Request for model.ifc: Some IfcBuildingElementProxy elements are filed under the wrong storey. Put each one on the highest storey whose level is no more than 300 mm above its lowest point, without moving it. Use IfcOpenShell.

First a look at what the model holds.

```python
import ifcopenshell
import ifcopenshell.util.element
import ifcopenshell.util.placement

model = ifcopenshell.open("model.ifc")
print(model.schema)
for storey in model.by_type("IfcBuildingStorey"):
    level = ifcopenshell.util.placement.get_storey_elevation(storey)
    count = sum(e.is_a("IfcBuildingElementProxy") for e in ifcopenshell.util.element.get_contained(storey))
    print(storey.id(), storey.Name, round(level, 3), count, sep=" | ")
```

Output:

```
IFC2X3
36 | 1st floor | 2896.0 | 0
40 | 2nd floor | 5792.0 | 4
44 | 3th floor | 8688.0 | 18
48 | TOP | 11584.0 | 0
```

```python
import ifcopenshell
import ifcopenshell.api.spatial
import ifcopenshell.geom
import ifcopenshell.util.element
import ifcopenshell.util.placement
import ifcopenshell.util.shape
import ifcopenshell.util.unit

model = ifcopenshell.open("model.ifc")
unit_scale = ifcopenshell.util.unit.calculate_unit_scale(model)
settings = ifcopenshell.geom.settings()

levels = sorted(
    ((ifcopenshell.util.placement.get_storey_elevation(s) * unit_scale, s) for s in model.by_type("IfcBuildingStorey")),
    key=lambda pair: pair[0],
)

for e in model.by_type("IfcBuildingElementProxy"):
    current = e.ContainedInStructure[0].RelatingStructure if e.ContainedInStructure else None
    if current is None or not current.is_a("IfcBuildingStorey"):
        continue
    shape = ifcopenshell.geom.create_shape(settings, e)
    bottom = ifcopenshell.util.shape.get_shape_bottom_elevation(shape, shape.geometry)
    below = [s for level, s in levels if level <= bottom + 0.3]
    storey = below[-1] if below else levels[0][1]
    if storey != current:
        # assign_container keeps the world position.
        ifcopenshell.api.spatial.assign_container(model, products=[e], relating_structure=storey)
        print(e.id(), current.Name, "->", storey.Name)

model.write("model_v2.ifc")
```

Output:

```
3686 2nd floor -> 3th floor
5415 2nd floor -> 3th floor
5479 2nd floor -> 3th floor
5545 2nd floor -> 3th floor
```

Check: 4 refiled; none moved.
